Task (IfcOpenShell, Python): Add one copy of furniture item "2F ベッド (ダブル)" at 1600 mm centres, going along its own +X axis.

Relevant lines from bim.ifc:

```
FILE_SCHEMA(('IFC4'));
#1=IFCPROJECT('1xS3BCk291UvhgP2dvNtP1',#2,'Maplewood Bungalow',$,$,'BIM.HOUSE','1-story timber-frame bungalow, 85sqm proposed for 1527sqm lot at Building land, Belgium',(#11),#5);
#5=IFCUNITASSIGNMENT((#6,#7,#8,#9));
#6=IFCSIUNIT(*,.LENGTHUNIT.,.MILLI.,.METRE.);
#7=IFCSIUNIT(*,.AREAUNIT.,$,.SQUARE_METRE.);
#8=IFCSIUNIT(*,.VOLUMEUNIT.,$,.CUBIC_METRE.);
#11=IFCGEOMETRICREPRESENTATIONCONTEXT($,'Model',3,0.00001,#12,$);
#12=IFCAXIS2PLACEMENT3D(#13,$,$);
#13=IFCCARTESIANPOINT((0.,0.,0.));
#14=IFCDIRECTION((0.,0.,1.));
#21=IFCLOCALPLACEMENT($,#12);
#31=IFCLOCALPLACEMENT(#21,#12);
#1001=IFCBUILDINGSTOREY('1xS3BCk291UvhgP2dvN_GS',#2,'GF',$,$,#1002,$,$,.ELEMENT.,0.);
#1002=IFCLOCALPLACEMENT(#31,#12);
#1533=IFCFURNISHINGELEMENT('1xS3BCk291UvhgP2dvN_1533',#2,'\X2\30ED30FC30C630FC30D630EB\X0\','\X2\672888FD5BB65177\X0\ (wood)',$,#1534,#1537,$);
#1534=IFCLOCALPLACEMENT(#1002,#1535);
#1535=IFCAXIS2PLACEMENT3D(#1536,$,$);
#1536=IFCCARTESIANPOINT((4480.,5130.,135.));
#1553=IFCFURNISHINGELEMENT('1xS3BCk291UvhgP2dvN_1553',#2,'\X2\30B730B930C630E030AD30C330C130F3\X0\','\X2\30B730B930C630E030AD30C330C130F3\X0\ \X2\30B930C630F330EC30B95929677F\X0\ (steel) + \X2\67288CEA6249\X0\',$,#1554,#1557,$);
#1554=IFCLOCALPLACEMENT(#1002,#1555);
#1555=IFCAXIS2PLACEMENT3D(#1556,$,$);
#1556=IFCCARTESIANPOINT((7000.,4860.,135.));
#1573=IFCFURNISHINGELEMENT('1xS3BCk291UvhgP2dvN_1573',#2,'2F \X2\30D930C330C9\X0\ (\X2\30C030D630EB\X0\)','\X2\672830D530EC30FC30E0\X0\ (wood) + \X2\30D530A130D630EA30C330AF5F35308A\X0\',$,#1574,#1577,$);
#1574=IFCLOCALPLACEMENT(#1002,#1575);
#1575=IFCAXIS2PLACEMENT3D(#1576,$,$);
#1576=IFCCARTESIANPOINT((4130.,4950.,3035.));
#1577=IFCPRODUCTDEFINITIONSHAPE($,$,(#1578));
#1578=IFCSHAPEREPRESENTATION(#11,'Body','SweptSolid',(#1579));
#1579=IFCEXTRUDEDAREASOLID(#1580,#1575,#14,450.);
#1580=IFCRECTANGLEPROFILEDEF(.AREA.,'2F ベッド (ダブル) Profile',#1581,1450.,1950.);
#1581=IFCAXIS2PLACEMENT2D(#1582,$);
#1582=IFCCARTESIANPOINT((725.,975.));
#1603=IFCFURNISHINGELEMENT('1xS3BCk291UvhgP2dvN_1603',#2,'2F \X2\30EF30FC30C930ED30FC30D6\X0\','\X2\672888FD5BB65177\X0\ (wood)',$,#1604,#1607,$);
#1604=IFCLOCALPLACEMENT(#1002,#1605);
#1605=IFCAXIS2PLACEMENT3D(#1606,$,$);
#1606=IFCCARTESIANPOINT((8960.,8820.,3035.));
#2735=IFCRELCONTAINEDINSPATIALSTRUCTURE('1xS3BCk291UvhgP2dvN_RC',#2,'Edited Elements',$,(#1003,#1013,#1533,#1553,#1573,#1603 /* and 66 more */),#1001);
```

```python
import ifcopenshell
import ifcopenshell.api.geometry
import ifcopenshell.api.root
import ifcopenshell.util.element
import ifcopenshell.util.placement
import ifcopenshell.util.unit

model = ifcopenshell.open("bim.ifc")
unit_scale = ifcopenshell.util.unit.calculate_unit_scale(model)


def reuse_history(source, copy):
    """copy_class also copies each property set's owner history, people and application; keep the originals."""
    for rel in copy.IsDefinedBy:
        if rel.is_a("IfcRelDefinesByProperties") and (history := rel.RelatingPropertyDefinition.OwnerHistory):
            rel.RelatingPropertyDefinition.OwnerHistory = source.OwnerHistory
            ifcopenshell.util.element.remove_deep2(model, history)


source = model.by_guid("1xS3BCk291UvhgP2dvN_1573")
base = ifcopenshell.util.placement.get_local_placement(source.ObjectPlacement)
step = base[:3, 0] * 1.6 / unit_scale

for i in range(1, 2):
    copy = ifcopenshell.api.root.copy_class(model, product=source)
    copy.Representation = ifcopenshell.util.element.copy_deep(
        model, source.Representation, exclude=["IfcGeometricRepresentationContext", "IfcRepresentationMap"]
    )
    reuse_history(source, copy)
    matrix = base.copy()
    matrix[:3, 3] += i * step
    print("added at", matrix[:3, 3].round(3) + 0.0)
    ifcopenshell.api.geometry.edit_object_placement(model, product=copy, matrix=matrix, is_si=False)

model.write("bim-out.ifc")
```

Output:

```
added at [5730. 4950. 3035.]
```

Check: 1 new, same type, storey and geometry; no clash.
